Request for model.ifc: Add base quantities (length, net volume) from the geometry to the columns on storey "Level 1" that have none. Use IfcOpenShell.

First a look at what the model holds.

```python
import ifcopenshell
import ifcopenshell.util.element
import ifcopenshell.util.unit

model = ifcopenshell.open("model.ifc")
print(model.schema)
for unit_type in ("LENGTHUNIT", "AREAUNIT", "VOLUMEUNIT"):
    print(unit_type, ifcopenshell.util.unit.calculate_unit_scale(model, unit_type))
storey = next(s for s in model.by_type("IfcBuildingStorey") if s.Name == "Level 1")
columns = [e for e in ifcopenshell.util.element.get_decomposition(storey) if e.is_a("IfcColumn")]
for e in sorted(columns, key=lambda e: e.id()):
    print(e.id(), e.is_a(), e.Name, list(ifcopenshell.util.element.get_psets(e, qtos_only=True)), sep=" | ")
```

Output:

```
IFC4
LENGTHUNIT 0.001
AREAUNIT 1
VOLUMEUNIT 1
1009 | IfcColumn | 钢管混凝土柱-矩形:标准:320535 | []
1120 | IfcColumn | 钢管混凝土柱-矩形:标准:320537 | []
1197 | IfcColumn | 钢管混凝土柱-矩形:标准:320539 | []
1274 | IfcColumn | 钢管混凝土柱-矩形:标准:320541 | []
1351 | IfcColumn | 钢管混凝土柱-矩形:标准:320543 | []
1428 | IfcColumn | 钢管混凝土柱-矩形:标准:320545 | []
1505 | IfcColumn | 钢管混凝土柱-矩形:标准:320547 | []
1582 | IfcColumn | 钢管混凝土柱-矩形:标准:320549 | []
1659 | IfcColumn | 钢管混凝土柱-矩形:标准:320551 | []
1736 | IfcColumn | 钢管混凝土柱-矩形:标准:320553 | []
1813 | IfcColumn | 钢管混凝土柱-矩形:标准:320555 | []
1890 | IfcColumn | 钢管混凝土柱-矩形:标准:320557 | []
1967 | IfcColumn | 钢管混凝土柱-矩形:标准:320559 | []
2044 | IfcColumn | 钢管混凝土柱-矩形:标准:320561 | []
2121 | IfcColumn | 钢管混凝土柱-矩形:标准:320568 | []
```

```python
import ifcopenshell
import ifcopenshell.api.pset
import ifcopenshell.geom
import ifcopenshell.util.element
import ifcopenshell.util.shape
import ifcopenshell.util.unit

model = ifcopenshell.open("model.ifc")
unit_scale = ifcopenshell.util.unit.calculate_unit_scale(model)
volume_scale = ifcopenshell.util.unit.calculate_unit_scale(model, "VOLUMEUNIT")
settings = ifcopenshell.geom.settings()

storey = next(s for s in model.by_type("IfcBuildingStorey") if s.Name == "Level 1")
columns = [e for e in ifcopenshell.util.element.get_decomposition(storey) if e.is_a("IfcColumn")]

for e in sorted(columns, key=lambda e: e.id()):
    if ifcopenshell.util.element.get_psets(e, qtos_only=True, should_inherit=False):
        continue
    # Geometry comes back in metres, in the element's own axes.
    shape = ifcopenshell.geom.create_shape(settings, e)
    values = {
        "Length": ifcopenshell.util.shape.get_z(shape.geometry) / unit_scale,
        "NetVolume": ifcopenshell.util.shape.get_volume(shape.geometry) / volume_scale,
    }
    qto = ifcopenshell.api.pset.add_qto(model, product=e, name="Qto_ColumnBaseQuantities")
    ifcopenshell.api.pset.edit_qto(model, qto=qto, properties=values)
    print(e.id(), {k: round(v, 3) for k, v in values.items()})

model.write("model_rev.ifc")
```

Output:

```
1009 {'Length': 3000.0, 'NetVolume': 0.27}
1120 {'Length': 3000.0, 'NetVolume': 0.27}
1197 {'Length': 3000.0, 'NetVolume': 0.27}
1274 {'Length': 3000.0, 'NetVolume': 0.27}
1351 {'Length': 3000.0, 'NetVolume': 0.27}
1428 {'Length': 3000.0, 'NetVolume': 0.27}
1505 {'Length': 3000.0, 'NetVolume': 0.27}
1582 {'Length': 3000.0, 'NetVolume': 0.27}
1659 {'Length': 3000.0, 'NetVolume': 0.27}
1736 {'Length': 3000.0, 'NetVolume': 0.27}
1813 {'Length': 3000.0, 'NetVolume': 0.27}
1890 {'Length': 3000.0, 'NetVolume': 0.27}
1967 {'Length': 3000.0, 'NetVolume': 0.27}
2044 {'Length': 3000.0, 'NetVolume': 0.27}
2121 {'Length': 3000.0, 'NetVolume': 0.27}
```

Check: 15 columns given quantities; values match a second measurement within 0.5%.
